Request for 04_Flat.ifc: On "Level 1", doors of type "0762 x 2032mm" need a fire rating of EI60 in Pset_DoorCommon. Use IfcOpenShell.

First a look at what the model holds.

```python
import ifcopenshell
import ifcopenshell.util.element

model = ifcopenshell.open("04_Flat.ifc")
print(model.schema)
storey = next(s for s in model.by_type("IfcBuildingStorey") if s.Name == "Level 1")
doors = [e for e in ifcopenshell.util.element.get_decomposition(storey) if e.is_a("IfcDoor")]
seen = {}
for e in doors:
    element_type = ifcopenshell.util.element.get_type(e)
    key = (element_type.Name if element_type != e and element_type else None, ifcopenshell.util.element.get_pset(e, "Pset_DoorCommon", "FireRating"))
    seen[key] = seen.get(key, 0) + 1
for (name, value), count in sorted(seen.items(), key=str):
    print(count, "x", name, "|", value)
```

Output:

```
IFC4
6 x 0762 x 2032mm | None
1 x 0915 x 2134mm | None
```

```python
import ifcopenshell
import ifcopenshell.api.pset
import ifcopenshell.util.element

model = ifcopenshell.open("04_Flat.ifc")

storey = next(s for s in model.by_type("IfcBuildingStorey") if s.Name == "Level 1")
doors = [e for e in ifcopenshell.util.element.get_decomposition(storey) if e.is_a("IfcDoor")]

count = 0
for e in doors:
    element_type = ifcopenshell.util.element.get_type(e)
    if element_type in (None, e) or element_type.Name != "0762 x 2032mm":
        continue
    # add_pset returns the element's existing set when there is one.
    pset = ifcopenshell.api.pset.add_pset(model, product=e, name="Pset_DoorCommon")
    ifcopenshell.api.pset.edit_pset(model, pset=pset, properties={"FireRating": "EI60"})
    count += 1

print(count, "doors updated")

model.write("04_Flat_updated.ifc")
```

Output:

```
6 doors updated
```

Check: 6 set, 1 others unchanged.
